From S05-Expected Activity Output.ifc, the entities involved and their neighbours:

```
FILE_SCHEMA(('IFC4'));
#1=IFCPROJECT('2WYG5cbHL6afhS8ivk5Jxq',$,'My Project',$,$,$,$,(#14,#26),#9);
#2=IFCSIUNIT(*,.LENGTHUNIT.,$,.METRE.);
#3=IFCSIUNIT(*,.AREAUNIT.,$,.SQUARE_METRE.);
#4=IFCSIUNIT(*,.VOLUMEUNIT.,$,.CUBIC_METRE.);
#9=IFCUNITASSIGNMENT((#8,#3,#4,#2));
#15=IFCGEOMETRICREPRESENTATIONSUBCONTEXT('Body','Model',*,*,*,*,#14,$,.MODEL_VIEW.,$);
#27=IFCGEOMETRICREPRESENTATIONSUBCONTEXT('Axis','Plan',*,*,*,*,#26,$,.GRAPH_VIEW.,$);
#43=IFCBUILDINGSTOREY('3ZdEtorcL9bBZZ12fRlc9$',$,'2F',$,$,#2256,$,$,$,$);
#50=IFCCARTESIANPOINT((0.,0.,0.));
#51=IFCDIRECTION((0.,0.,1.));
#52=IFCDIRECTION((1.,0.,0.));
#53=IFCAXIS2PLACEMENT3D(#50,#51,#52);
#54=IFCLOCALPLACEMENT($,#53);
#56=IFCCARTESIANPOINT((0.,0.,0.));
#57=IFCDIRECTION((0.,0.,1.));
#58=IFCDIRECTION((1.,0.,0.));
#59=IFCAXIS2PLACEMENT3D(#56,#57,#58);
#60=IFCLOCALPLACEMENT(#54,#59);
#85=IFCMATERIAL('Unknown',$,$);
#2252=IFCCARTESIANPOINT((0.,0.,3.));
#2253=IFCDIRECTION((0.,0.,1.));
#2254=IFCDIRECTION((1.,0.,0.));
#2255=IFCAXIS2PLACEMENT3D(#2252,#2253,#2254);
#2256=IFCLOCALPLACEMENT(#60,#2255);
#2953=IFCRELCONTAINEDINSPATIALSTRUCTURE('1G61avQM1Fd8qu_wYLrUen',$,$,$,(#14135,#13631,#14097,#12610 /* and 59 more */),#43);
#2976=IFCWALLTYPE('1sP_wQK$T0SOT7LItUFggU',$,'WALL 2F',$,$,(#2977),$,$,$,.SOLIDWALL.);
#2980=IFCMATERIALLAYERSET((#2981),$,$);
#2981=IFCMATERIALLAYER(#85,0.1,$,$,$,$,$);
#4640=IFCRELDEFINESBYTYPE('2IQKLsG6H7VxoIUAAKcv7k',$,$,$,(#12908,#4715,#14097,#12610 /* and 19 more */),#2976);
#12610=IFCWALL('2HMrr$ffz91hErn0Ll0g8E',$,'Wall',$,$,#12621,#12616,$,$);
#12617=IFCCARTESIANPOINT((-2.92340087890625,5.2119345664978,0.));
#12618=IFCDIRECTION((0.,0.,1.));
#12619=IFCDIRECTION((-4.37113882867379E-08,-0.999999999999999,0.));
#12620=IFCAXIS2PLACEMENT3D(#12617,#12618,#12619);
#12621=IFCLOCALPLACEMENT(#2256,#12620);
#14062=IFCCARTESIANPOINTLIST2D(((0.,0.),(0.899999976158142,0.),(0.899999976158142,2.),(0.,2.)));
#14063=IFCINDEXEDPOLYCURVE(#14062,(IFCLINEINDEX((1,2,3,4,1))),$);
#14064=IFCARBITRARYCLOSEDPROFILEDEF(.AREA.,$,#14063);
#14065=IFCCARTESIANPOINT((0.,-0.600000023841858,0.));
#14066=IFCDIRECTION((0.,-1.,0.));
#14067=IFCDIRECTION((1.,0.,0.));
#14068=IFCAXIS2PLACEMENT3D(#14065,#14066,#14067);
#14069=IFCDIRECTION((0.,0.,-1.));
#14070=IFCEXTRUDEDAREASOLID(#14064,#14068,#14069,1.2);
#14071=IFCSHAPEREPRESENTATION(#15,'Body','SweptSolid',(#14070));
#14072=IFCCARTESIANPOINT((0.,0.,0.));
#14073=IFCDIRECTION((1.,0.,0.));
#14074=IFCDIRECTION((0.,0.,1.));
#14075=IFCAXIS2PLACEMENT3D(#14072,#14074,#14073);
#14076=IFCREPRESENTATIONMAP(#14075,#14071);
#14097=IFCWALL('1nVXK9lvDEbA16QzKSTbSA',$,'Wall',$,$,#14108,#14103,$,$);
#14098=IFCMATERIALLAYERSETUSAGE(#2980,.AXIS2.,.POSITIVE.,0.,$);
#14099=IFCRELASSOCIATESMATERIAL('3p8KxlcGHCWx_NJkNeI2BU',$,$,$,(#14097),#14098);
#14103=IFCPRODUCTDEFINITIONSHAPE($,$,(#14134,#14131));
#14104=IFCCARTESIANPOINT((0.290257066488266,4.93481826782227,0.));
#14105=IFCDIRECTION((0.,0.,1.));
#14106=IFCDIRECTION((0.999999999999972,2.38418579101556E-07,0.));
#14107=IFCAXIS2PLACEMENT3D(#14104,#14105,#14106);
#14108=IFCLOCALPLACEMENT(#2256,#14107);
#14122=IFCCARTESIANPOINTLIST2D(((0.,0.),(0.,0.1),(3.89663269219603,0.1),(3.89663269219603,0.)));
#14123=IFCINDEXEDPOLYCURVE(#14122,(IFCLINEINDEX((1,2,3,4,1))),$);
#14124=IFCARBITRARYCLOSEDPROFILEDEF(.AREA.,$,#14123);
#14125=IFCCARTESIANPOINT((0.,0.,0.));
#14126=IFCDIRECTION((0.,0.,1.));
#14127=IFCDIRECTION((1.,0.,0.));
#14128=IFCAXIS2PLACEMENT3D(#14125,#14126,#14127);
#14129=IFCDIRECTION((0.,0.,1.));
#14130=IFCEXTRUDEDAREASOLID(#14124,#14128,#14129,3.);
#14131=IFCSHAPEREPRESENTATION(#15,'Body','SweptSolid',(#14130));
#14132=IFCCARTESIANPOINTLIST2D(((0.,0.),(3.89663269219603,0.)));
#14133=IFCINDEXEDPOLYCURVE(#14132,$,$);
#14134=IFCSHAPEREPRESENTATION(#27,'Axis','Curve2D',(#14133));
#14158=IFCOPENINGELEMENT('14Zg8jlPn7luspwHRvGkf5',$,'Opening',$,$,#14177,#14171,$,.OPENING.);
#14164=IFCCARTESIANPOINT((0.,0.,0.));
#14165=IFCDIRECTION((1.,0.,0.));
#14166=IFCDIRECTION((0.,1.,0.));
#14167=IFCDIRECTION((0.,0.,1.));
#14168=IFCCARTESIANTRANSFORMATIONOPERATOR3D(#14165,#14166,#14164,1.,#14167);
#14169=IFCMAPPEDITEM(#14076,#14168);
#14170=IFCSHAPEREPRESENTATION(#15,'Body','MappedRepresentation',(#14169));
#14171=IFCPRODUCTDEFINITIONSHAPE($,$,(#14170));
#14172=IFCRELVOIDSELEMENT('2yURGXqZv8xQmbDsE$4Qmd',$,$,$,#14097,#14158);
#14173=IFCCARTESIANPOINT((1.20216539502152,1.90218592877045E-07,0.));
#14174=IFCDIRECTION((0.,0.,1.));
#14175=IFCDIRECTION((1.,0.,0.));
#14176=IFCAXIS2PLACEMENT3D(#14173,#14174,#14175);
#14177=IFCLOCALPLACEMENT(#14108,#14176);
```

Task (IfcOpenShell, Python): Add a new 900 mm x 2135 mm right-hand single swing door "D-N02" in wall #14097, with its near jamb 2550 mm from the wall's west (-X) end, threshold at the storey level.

```python
import numpy as np
import ifcopenshell
import ifcopenshell.api.feature
import ifcopenshell.api.geometry
import ifcopenshell.api.root
import ifcopenshell.api.spatial
import ifcopenshell.geom
import ifcopenshell.util.element
import ifcopenshell.util.placement
import ifcopenshell.util.representation
import ifcopenshell.util.shape
import ifcopenshell.util.unit

model = ifcopenshell.open("S05-Expected Activity Output.ifc")
unit_scale = ifcopenshell.util.unit.calculate_unit_scale(model)
settings = ifcopenshell.geom.settings()


def volume(element):
    """Net volume in cubic metres, openings subtracted."""
    shape = ifcopenshell.geom.create_shape(settings, element)
    return ifcopenshell.util.shape.get_volume(shape.geometry)


wall = model.by_id(14097)
storey = ifcopenshell.util.element.get_container(wall, ifc_class="IfcBuildingStorey")
context = ifcopenshell.util.representation.get_context(model, "Model", "Body", "MODEL_VIEW")
before = volume(wall)

width, height, from_end, sill = 0.9, 2.135, 2.55, 0.0  # metres

# The wall runs along its own X axis, and the end named is its -X end.
wall_shape = ifcopenshell.geom.create_shape(settings, wall)
x, y, z = ifcopenshell.util.shape.get_vertices(wall_shape.geometry).T
start = x.min() + from_end
face, thickness = float(y.min()), float(y.max() - y.min())
wall_matrix = ifcopenshell.util.placement.get_local_placement(wall.ObjectPlacement)
level = ifcopenshell.util.placement.get_local_placement(storey.ObjectPlacement)[2, 3]


def in_wall(x, y):
    """Placement at x, y metres in the wall's axes, at sill height."""
    matrix = wall_matrix.copy()
    matrix[:, 3] = wall_matrix @ np.array([x / unit_scale, y / unit_scale, 0.0, 1.0])
    matrix[2, 3] = level + sill / unit_scale
    return matrix


# Opening: a box that overshoots both wall faces by 50 mm.
opening = ifcopenshell.api.root.create_entity(model, ifc_class="IfcOpeningElement", predefined_type="OPENING")
box = ifcopenshell.api.geometry.add_wall_representation(
    model, context=context, length=width, height=height, thickness=thickness + 0.1
)
ifcopenshell.api.geometry.assign_representation(model, product=opening, representation=box)
ifcopenshell.api.geometry.edit_object_placement(model, product=opening, matrix=in_wall(start, face - 0.05), is_si=False)
ifcopenshell.api.feature.add_feature(model, feature=opening, element=wall)

door = ifcopenshell.api.root.create_entity(model, ifc_class="IfcDoor", name="D-N02", predefined_type="DOOR")
door.OverallWidth, door.OverallHeight = width / unit_scale, height / unit_scale
door.OperationType = "SINGLE_SWING_RIGHT"
body = ifcopenshell.api.geometry.add_door_representation(
    model,
    context=context,
    overall_width=door.OverallWidth,
    overall_height=door.OverallHeight,
    operation_type="SINGLE_SWING_RIGHT",
    lining_properties={"LiningDepth": thickness / unit_scale, "ThresholdDepth": thickness / unit_scale},
)
ifcopenshell.api.geometry.assign_representation(model, product=door, representation=body)
ifcopenshell.api.spatial.assign_container(model, products=[door], relating_structure=storey)
ifcopenshell.api.feature.add_filling(model, opening=opening, element=door)

# The lining spans the wall, so the door starts at the wall face.
ifcopenshell.api.geometry.edit_object_placement(model, product=door, matrix=in_wall(start, face), is_si=False)

after = volume(wall)

print(f"wall volume {before:.3f} -> {after:.3f} m3")

model.write("S05-Expected Activity Output_updated.ifc")
```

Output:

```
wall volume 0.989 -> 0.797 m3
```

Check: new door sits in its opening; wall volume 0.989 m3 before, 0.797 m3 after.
